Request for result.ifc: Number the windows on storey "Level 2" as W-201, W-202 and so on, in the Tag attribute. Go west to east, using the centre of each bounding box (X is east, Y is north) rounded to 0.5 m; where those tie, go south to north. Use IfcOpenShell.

First a look at what the model holds.

```python
import ifcopenshell
import ifcopenshell.util.element
import ifcopenshell.util.placement

model = ifcopenshell.open("result.ifc")
print(model.schema)
storey = next(s for s in model.by_type("IfcBuildingStorey") if s.Name == "Level 2")
windows = [e for e in ifcopenshell.util.element.get_decomposition(storey) if e.is_a("IfcWindow")]
for e in sorted(windows, key=lambda e: e.id()):
    origin = ifcopenshell.util.placement.get_local_placement(e.ObjectPlacement)[:3, 3]
    print(e.id(), e.Tag, e.Name, origin.round(2) + 0.0, sep=" | ")
```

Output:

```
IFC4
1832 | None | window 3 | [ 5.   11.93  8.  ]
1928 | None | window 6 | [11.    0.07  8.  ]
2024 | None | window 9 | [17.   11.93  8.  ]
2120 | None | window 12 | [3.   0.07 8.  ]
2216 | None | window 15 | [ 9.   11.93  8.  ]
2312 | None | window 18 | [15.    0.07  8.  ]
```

```python
import ifcopenshell
import ifcopenshell.geom
import ifcopenshell.util.element
import ifcopenshell.util.shape

model = ifcopenshell.open("result.ifc")
settings = ifcopenshell.geom.settings()
settings.set("use-world-coords", True)


def centre(element):
    shape = ifcopenshell.geom.create_shape(settings, element)
    return ifcopenshell.util.shape.get_bbox_centroid(shape.geometry)


storey = next(s for s in model.by_type("IfcBuildingStorey") if s.Name == "Level 2")
windows = [e for e in ifcopenshell.util.element.get_decomposition(storey) if e.is_a("IfcWindow")]

# Insertion points can sit at a corner or the storey origin, so sort by the geometry (in metres).
centres = {e: centre(e) for e in windows}
windows.sort(key=lambda e: (round(centres[e][0] / 0.5), centres[e][1]))

for i, e in enumerate(windows, start=1):
    number = f"W-2{i:02d}"
    e.Tag = number
    print(e.id(), number)

model.write("result_v2.ifc")
```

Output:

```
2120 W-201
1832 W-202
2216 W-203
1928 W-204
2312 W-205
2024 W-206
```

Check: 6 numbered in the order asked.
